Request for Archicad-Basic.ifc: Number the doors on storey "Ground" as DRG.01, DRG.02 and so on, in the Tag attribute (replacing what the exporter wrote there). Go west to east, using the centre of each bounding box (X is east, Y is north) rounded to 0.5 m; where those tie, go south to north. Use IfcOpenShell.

First a look at what the model holds.

```python
import ifcopenshell
import ifcopenshell.util.element
import ifcopenshell.util.placement

model = ifcopenshell.open("Archicad-Basic.ifc")
print(model.schema)
storey = next(s for s in model.by_type("IfcBuildingStorey") if s.Name == "Ground")
doors = [e for e in ifcopenshell.util.element.get_decomposition(storey) if e.is_a("IfcDoor")]
for e in sorted(doors, key=lambda e: e.id()):
    origin = ifcopenshell.util.placement.get_local_placement(e.ObjectPlacement)[:3, 3]
    print(e.id(), e.Tag, e.Name, origin.round(2) + 0.0, sep=" | ")
```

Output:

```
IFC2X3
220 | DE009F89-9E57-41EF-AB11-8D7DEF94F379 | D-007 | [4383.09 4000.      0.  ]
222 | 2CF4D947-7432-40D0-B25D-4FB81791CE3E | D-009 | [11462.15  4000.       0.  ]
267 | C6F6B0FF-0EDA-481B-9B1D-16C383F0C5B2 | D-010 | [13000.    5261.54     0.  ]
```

```python
import ifcopenshell
import ifcopenshell.geom
import ifcopenshell.util.element
import ifcopenshell.util.shape

model = ifcopenshell.open("Archicad-Basic.ifc")
settings = ifcopenshell.geom.settings()
settings.set("use-world-coords", True)


def centre(element):
    shape = ifcopenshell.geom.create_shape(settings, element)
    return ifcopenshell.util.shape.get_bbox_centroid(shape.geometry)


storey = next(s for s in model.by_type("IfcBuildingStorey") if s.Name == "Ground")
doors = [e for e in ifcopenshell.util.element.get_decomposition(storey) if e.is_a("IfcDoor")]

# Insertion points can sit at a corner or the storey origin, so sort by the geometry (in metres).
centres = {e: centre(e) for e in doors}
doors.sort(key=lambda e: (round(centres[e][0] / 0.5), centres[e][1]))

for i, e in enumerate(doors, start=1):
    number = f"DRG.{i:02d}"
    e.Tag = number
    print(e.id(), number)

model.write("Archicad-Basic_rev.ifc")
```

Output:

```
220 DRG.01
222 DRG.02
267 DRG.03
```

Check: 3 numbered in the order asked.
